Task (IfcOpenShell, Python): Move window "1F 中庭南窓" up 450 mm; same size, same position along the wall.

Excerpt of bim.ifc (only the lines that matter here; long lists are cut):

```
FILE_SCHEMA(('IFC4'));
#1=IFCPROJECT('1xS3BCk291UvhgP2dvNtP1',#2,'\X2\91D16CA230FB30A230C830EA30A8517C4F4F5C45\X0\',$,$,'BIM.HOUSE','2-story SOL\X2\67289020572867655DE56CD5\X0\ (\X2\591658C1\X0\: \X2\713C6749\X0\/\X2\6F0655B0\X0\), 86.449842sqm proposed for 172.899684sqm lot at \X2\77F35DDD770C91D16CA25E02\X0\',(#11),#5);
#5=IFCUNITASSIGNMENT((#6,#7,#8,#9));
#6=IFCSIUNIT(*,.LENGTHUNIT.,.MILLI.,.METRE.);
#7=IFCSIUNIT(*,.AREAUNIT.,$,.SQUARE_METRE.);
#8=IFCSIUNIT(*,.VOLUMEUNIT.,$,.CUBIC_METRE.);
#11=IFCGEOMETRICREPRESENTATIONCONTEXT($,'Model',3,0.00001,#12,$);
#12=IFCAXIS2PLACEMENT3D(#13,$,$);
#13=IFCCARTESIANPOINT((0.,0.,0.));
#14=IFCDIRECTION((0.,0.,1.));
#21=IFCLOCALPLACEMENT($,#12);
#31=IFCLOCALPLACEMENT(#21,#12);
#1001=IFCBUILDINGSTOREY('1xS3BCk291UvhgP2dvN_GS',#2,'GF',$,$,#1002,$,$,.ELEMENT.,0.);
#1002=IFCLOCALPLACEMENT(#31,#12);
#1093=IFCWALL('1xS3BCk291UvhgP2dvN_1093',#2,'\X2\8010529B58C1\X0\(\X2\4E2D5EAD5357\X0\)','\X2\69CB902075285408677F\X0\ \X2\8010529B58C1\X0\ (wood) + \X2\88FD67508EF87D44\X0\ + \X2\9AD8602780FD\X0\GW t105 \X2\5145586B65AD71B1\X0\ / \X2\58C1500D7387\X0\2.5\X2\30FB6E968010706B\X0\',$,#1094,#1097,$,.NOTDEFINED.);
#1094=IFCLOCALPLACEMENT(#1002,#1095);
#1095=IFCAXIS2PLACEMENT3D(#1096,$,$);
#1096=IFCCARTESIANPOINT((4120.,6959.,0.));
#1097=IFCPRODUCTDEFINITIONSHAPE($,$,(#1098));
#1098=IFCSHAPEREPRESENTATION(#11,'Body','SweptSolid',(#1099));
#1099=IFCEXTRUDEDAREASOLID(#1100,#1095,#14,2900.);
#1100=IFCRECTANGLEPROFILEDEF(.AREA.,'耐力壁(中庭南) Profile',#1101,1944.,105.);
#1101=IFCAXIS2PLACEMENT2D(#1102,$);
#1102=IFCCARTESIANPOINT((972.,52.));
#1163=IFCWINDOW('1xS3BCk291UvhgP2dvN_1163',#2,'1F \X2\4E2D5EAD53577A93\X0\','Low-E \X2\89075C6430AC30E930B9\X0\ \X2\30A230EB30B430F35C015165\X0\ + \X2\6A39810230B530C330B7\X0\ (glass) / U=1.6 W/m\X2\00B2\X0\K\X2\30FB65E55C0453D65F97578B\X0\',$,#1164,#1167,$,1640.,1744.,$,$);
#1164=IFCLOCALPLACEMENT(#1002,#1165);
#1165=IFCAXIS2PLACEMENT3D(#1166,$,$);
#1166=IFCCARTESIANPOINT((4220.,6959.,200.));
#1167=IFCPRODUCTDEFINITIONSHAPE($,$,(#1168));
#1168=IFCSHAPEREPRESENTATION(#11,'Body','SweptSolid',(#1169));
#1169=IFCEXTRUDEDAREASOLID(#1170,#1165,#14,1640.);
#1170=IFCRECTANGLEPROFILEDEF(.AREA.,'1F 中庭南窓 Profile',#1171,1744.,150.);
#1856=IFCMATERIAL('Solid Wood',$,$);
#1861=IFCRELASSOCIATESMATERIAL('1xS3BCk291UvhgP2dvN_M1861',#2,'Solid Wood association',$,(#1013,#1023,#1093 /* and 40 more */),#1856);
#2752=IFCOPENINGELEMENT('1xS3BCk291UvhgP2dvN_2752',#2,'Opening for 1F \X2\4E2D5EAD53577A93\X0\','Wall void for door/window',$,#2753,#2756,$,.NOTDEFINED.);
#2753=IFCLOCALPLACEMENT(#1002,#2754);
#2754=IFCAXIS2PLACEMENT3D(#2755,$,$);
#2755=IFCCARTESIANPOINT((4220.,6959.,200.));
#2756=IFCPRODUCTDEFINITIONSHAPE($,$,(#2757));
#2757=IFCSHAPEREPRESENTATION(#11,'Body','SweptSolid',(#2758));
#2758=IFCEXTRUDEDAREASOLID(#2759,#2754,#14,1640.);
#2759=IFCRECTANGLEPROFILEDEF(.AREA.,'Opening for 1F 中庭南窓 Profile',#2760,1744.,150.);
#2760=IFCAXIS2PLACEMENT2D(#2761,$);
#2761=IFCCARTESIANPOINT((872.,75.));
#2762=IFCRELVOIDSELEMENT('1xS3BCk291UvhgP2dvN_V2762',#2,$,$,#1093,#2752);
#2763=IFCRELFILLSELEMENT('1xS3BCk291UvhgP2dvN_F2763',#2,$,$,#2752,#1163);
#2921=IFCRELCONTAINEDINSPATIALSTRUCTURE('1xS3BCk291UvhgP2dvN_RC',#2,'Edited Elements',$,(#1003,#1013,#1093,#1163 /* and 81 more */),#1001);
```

```python
import numpy as np
import ifcopenshell
import ifcopenshell.api.geometry
import ifcopenshell.util.placement
import ifcopenshell.util.unit

model = ifcopenshell.open("bim.ifc")
unit_scale = ifcopenshell.util.unit.calculate_unit_scale(model)

window = model.by_guid("1xS3BCk291UvhgP2dvN_1163")
opening = window.FillsVoids[0].RelatingOpeningElement
dz = 0.45 / unit_scale

shift = np.array([0.0, 0.0, dz])
# The window is not placed relative to its opening, so move both.
for product in (opening, window):
    matrix = ifcopenshell.util.placement.get_local_placement(product.ObjectPlacement)
    matrix[:3, 3] += shift
    ifcopenshell.api.geometry.edit_object_placement(model, product=product, matrix=matrix, is_si=False)

print(f"moved by {dz * unit_scale:+.3f} m")

model.write("bim_updated.ifc")
```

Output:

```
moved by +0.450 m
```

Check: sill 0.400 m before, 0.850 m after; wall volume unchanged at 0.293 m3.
